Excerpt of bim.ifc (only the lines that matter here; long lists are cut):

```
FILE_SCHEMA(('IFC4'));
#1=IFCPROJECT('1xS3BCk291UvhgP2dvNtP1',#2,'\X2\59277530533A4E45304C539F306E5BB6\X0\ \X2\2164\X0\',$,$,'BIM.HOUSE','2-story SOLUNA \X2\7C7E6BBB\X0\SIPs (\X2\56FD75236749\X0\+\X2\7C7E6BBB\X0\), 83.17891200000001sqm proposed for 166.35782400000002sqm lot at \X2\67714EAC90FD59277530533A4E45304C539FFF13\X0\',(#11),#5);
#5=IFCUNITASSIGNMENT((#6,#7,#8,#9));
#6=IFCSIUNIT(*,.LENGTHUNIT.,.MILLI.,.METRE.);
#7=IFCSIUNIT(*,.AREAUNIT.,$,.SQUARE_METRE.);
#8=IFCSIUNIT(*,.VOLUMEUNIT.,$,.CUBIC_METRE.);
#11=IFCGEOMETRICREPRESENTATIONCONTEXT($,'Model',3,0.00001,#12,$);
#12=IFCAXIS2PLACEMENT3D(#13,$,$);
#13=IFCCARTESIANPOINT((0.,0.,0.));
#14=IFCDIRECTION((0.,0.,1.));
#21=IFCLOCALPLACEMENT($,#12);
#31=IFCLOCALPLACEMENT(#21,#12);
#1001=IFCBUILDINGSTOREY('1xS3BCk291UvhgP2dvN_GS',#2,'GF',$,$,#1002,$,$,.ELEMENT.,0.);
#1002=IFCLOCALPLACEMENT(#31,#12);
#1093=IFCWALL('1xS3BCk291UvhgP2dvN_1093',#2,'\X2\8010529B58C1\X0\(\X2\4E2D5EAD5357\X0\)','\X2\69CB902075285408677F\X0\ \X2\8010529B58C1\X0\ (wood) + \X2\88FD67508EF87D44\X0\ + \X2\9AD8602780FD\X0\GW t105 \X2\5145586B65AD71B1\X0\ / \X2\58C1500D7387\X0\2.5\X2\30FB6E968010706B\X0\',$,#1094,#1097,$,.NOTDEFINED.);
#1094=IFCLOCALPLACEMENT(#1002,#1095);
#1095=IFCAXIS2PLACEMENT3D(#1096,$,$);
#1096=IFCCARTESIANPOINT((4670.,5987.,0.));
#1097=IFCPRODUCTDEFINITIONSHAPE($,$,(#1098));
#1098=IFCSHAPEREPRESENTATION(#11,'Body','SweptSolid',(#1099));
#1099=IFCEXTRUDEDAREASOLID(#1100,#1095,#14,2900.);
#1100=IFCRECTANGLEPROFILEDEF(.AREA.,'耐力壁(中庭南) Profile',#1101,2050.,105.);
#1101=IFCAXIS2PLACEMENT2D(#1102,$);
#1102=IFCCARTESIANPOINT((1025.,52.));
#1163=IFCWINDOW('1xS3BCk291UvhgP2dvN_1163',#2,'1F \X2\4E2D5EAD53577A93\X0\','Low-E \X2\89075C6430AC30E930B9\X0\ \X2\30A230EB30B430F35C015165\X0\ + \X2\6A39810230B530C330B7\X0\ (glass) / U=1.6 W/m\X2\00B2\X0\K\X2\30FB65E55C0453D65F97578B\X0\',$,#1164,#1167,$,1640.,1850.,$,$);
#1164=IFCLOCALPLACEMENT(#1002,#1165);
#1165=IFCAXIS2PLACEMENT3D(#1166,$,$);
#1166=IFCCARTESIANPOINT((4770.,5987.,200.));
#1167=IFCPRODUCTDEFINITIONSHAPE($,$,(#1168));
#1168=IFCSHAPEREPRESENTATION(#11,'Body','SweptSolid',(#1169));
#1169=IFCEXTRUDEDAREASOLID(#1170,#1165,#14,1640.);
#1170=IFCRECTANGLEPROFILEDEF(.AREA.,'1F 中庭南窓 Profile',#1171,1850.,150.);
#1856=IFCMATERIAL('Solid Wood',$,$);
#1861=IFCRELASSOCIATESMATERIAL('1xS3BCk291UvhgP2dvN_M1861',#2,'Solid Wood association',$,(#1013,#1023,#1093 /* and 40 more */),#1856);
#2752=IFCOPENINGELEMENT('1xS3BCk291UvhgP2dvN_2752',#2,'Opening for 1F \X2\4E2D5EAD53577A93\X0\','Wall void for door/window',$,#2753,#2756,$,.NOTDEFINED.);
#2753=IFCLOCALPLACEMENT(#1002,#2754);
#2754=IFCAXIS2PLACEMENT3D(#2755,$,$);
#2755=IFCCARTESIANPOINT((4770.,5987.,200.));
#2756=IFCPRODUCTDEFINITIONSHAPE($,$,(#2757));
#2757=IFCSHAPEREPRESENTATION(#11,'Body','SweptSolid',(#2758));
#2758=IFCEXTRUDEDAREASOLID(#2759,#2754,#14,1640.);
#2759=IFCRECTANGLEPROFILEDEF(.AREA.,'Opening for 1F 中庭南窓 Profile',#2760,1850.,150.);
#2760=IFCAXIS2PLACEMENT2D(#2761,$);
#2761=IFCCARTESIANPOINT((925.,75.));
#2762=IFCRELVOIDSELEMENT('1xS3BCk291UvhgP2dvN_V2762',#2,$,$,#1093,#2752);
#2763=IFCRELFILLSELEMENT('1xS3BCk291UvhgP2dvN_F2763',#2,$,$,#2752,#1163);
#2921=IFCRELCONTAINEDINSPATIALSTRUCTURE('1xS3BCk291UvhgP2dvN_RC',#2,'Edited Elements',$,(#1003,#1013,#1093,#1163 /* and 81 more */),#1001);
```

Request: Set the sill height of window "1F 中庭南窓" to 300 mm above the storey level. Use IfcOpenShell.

```python
import numpy as np
import ifcopenshell
import ifcopenshell.api.geometry
import ifcopenshell.geom
import ifcopenshell.util.element
import ifcopenshell.util.placement
import ifcopenshell.util.shape
import ifcopenshell.util.unit

model = ifcopenshell.open("bim.ifc")
unit_scale = ifcopenshell.util.unit.calculate_unit_scale(model)

window = model.by_guid("1xS3BCk291UvhgP2dvN_1163")
opening = window.FillsVoids[0].RelatingOpeningElement
storey = ifcopenshell.util.element.get_container(window, ifc_class="IfcBuildingStorey")
level = ifcopenshell.util.placement.get_local_placement(storey.ObjectPlacement)[2, 3]

# The opening's origin need not be at the sill, so measure its lowest point.
shape = ifcopenshell.geom.create_shape(ifcopenshell.geom.settings(), opening)
bottom = ifcopenshell.util.shape.get_shape_bottom_elevation(shape, shape.geometry) / unit_scale
dz = level + 0.3 / unit_scale - bottom

shift = np.array([0.0, 0.0, dz])
# The window is not placed relative to its opening, so move both.
for product in (opening, window):
    matrix = ifcopenshell.util.placement.get_local_placement(product.ObjectPlacement)
    matrix[:3, 3] += shift
    ifcopenshell.api.geometry.edit_object_placement(model, product=product, matrix=matrix, is_si=False)

print(f"moved by {dz * unit_scale:+.3f} m")

model.write("bim_updated.ifc")
```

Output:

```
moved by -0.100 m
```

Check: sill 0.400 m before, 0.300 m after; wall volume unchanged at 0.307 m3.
